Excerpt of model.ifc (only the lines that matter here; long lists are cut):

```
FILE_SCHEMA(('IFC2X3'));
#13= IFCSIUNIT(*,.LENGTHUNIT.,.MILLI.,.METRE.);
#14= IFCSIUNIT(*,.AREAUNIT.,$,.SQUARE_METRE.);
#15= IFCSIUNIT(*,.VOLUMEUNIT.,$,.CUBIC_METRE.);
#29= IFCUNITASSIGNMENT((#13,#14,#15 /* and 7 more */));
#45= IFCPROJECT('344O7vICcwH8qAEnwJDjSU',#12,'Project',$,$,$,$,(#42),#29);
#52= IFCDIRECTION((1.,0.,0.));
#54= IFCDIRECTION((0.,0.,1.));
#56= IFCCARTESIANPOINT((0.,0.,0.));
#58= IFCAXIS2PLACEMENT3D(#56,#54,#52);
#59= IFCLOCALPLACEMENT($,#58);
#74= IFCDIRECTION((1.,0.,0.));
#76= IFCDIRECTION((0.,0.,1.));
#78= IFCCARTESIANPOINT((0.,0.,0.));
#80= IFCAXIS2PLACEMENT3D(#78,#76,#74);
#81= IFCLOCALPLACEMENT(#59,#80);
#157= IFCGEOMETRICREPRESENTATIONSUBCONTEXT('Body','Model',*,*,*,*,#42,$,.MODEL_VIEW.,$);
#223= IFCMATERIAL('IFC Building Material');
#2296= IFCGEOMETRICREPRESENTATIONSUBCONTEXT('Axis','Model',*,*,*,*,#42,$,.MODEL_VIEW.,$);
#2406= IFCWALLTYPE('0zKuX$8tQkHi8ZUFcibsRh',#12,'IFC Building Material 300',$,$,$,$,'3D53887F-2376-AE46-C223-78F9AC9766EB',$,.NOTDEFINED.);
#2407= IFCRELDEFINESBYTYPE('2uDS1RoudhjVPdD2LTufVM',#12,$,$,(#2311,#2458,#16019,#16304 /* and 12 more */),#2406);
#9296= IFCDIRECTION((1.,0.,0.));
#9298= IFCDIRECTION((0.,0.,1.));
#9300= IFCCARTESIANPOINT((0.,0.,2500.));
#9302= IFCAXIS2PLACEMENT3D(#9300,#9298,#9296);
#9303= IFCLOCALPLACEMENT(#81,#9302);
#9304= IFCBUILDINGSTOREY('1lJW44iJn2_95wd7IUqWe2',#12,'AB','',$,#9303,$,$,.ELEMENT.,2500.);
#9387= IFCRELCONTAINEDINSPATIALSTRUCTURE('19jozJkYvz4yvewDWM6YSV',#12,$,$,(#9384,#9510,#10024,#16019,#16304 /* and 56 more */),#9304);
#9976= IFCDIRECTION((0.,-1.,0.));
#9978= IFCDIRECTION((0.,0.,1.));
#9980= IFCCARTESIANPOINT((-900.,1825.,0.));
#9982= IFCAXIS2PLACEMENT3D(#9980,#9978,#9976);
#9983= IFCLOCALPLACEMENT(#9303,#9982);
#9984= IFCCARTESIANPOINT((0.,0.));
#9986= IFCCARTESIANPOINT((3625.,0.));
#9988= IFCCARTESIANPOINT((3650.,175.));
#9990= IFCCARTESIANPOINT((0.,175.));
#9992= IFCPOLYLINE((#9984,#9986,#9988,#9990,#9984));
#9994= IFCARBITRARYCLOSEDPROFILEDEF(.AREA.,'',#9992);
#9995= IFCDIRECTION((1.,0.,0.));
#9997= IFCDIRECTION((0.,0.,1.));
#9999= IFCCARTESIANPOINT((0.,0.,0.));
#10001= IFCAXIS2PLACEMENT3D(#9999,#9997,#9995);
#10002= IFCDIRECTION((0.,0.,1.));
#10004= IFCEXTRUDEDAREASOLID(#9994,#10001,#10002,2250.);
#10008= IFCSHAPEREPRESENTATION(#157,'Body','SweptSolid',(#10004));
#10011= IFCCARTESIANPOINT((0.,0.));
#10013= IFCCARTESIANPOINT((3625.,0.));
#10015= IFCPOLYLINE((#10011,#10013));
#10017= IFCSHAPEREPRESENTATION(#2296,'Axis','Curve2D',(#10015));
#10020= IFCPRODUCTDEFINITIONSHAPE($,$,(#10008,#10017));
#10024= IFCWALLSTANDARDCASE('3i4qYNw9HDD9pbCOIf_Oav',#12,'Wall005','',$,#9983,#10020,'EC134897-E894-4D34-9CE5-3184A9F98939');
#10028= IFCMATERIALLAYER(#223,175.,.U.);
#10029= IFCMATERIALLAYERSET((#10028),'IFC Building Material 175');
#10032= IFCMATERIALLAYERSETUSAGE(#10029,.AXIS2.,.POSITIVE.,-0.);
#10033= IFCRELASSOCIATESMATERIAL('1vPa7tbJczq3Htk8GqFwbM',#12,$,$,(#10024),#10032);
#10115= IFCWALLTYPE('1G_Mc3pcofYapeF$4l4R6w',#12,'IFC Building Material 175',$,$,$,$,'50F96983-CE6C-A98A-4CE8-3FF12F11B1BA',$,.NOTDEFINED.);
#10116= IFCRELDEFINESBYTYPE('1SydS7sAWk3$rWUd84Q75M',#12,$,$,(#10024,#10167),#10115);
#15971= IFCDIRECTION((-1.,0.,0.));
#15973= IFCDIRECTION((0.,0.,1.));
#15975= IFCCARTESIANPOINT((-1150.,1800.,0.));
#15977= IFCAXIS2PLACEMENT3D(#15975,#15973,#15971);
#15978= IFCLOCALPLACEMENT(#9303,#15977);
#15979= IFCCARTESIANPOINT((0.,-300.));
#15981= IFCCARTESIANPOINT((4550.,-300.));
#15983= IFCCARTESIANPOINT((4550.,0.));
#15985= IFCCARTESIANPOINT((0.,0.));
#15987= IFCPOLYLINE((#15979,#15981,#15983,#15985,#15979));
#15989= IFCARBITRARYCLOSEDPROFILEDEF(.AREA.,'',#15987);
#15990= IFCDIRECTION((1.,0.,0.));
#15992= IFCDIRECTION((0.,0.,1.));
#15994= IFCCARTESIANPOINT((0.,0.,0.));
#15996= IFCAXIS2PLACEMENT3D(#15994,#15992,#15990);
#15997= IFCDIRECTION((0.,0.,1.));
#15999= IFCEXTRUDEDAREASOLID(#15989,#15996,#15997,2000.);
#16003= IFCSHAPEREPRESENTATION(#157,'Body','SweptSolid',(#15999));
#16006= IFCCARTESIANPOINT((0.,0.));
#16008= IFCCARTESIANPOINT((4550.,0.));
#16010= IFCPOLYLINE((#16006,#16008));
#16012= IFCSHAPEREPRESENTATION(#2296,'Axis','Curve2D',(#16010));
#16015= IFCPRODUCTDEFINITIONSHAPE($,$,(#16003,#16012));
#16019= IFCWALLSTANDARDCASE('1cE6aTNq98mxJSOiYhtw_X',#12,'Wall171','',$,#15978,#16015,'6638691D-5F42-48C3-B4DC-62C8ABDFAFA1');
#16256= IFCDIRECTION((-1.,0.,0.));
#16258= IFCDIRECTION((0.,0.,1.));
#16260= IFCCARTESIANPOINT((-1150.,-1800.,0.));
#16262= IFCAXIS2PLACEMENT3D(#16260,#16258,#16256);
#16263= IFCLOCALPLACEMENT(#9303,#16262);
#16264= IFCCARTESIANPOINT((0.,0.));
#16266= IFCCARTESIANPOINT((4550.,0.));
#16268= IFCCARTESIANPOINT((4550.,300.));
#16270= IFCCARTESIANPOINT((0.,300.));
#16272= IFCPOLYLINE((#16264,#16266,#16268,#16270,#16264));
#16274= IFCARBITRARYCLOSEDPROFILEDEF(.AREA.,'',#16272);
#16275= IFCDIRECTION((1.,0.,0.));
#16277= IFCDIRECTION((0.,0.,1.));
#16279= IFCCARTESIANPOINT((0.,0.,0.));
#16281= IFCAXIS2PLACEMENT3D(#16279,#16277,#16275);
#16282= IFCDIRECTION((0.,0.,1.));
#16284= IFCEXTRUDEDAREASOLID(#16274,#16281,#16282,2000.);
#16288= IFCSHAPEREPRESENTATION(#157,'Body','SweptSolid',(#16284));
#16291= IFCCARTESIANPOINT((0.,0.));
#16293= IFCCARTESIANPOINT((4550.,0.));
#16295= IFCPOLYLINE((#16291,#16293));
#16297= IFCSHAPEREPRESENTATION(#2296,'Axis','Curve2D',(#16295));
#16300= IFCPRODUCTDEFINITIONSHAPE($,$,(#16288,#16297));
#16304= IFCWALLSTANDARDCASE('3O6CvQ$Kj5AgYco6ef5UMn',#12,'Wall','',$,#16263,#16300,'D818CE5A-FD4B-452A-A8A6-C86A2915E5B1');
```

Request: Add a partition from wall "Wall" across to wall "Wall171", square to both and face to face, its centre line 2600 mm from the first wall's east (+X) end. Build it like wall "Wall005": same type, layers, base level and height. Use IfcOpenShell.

```python
import numpy as np
import ifcopenshell
import ifcopenshell.api.geometry
import ifcopenshell.api.material
import ifcopenshell.api.pset
import ifcopenshell.api.root
import ifcopenshell.api.spatial
import ifcopenshell.api.type
import ifcopenshell.geom
import ifcopenshell.util.element
import ifcopenshell.util.placement
import ifcopenshell.util.representation
import ifcopenshell.util.shape
import ifcopenshell.util.unit

model = ifcopenshell.open("model.ifc")
unit_scale = ifcopenshell.util.unit.calculate_unit_scale(model)
settings = ifcopenshell.geom.settings()
settings.set("use-world-coords", True)

start_wall = model.by_guid("3O6CvQ$Kj5AgYco6ef5UMn")
end_wall = model.by_guid("1cE6aTNq98mxJSOiYhtw_X")
like = model.by_guid("3i4qYNw9HDD9pbCOIf_Oav")
matrix = ifcopenshell.util.placement.get_local_placement(start_wall.ObjectPlacement)
matrix[:3, 3] *= unit_scale


def extent(element):
    """Bounding box in the first wall's axes, in metres."""
    shape = ifcopenshell.geom.create_shape(settings, element)
    points = (ifcopenshell.util.shape.get_vertices(shape.geometry) - matrix[:3, 3]) @ matrix[:3, :3]
    return points.min(axis=0), points.max(axis=0)


y_start = extent(start_wall)[0][1]
y_end = extent(end_wall)[1][1]
like_min, like_max = extent(like)
length, height = float(abs(y_end - y_start)), float(like_max[2] - like_min[2])
layer_set = ifcopenshell.util.element.get_material(like, should_skip_usage=True)
thickness = sum(layer.LayerThickness for layer in layer_set.MaterialLayers) * unit_scale

wall = ifcopenshell.api.root.create_entity(model, ifc_class="IfcWallStandardCase", name="New partition")
storey = ifcopenshell.util.element.get_container(like)
ifcopenshell.api.spatial.assign_container(model, products=[wall], relating_structure=storey)
ifcopenshell.api.type.assign_type(
    model, related_objects=[wall], relating_type=ifcopenshell.util.element.get_type(like), should_map_representations=False
)
rel = ifcopenshell.api.material.assign_material(
    model, products=[wall], type="IfcMaterialLayerSetUsage", material=layer_set
)
rel.RelatingMaterial.OffsetFromReferenceLine = -thickness / 2 / unit_scale
pset = ifcopenshell.api.pset.add_pset(model, product=wall, name="Pset_WallCommon")
ifcopenshell.api.pset.edit_pset(model, pset=pset, properties={"IsExternal": False, "LoadBearing": False})

# The axis runs down the middle of the wall.
axis = ifcopenshell.api.geometry.add_axis_representation(
    model, context=ifcopenshell.util.representation.get_context(model, "Model", "Axis"), axis=[(0.0, 0.0), (length, 0.0)]
)
body = ifcopenshell.api.geometry.add_wall_representation(
    model,
    context=ifcopenshell.util.representation.get_context(model, "Model", "Body", "MODEL_VIEW"),
    length=length,
    height=height,
    thickness=thickness,
    offset=-thickness / 2,
)
for representation in (axis, body):
    ifcopenshell.api.geometry.assign_representation(model, product=wall, representation=representation)

placement = matrix @ ifcopenshell.util.placement.rotation(-90, "Z")
placement[:, 3] = matrix @ np.array([extent(start_wall)[0][0] + 2.6, y_start, like_min[2], 1.0])
ifcopenshell.api.geometry.edit_object_placement(model, product=wall, matrix=placement)

print(f"partition {length:.3f} m long, {height:.3f} m high, {thickness:.3f} m thick")

model.write("model-out.ifc")
```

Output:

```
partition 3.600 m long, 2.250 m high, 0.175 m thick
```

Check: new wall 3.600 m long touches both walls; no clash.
